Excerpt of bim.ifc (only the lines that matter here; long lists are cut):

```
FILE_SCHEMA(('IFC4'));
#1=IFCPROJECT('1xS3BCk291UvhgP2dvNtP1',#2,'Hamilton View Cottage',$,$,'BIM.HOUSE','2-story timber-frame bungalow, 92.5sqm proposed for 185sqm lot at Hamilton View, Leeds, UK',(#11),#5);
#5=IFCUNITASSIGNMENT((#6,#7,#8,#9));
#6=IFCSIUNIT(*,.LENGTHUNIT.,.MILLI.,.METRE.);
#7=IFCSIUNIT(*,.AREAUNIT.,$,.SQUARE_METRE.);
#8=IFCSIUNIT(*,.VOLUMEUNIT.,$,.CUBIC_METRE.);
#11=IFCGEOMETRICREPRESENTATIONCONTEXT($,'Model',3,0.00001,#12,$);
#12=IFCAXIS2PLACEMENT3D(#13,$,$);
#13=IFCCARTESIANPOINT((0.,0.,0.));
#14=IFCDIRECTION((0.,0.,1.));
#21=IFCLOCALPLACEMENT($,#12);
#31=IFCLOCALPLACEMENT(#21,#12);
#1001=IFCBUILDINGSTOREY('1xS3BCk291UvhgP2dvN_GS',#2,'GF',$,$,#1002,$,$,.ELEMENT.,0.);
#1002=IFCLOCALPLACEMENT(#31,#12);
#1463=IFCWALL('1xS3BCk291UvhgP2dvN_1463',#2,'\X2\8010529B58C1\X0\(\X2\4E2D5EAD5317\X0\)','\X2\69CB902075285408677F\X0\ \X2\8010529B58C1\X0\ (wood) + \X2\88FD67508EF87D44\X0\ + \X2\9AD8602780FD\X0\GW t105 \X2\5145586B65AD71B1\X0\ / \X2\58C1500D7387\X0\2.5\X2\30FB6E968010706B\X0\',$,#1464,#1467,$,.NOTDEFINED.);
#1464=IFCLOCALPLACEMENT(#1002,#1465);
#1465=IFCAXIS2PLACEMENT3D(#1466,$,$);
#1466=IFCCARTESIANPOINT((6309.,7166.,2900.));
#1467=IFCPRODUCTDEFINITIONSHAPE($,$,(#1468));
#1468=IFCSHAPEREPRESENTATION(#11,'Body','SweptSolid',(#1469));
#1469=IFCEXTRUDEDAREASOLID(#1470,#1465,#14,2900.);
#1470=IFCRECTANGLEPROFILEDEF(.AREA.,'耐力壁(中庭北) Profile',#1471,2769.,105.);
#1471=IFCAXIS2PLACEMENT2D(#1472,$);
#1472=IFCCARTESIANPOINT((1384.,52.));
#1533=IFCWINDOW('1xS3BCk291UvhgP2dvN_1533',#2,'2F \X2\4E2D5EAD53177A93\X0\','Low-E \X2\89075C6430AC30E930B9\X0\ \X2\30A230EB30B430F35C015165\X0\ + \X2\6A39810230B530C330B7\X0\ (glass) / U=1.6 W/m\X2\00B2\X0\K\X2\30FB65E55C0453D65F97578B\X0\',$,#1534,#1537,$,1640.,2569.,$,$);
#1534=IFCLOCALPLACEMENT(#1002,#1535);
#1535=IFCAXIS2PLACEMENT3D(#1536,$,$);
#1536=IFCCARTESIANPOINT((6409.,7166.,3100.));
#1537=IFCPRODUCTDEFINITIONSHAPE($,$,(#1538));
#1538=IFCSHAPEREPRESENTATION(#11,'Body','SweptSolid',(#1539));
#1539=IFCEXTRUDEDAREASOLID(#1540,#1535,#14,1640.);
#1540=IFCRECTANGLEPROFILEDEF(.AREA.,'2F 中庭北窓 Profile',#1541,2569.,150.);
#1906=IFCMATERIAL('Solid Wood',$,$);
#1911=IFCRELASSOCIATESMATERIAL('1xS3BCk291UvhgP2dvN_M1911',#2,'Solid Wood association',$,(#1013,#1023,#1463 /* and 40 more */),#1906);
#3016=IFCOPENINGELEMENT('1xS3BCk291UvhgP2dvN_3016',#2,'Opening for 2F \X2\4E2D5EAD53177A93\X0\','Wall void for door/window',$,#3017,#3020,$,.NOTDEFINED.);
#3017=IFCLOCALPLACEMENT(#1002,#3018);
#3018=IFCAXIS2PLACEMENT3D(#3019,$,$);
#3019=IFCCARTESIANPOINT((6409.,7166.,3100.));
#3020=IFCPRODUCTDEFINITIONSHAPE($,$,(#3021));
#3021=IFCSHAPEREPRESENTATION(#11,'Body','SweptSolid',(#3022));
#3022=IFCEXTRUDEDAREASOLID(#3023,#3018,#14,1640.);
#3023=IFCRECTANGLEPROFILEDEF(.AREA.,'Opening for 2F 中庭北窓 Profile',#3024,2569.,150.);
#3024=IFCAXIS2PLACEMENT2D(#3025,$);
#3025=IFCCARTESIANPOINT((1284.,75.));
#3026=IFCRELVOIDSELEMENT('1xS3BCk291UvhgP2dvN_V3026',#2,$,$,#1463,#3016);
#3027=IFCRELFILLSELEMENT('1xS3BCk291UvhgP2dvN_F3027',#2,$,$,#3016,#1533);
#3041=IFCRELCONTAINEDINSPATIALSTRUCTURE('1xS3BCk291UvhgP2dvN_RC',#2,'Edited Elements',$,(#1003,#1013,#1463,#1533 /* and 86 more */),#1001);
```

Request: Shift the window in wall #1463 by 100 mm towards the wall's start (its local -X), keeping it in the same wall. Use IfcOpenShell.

```python
import ifcopenshell
import ifcopenshell.api.geometry
import ifcopenshell.util.placement
import ifcopenshell.util.unit

model = ifcopenshell.open("bim.ifc")
unit_scale = ifcopenshell.util.unit.calculate_unit_scale(model)

window = model.by_id(1533)
opening = window.FillsVoids[0].RelatingOpeningElement
wall = opening.VoidsElements[0].RelatingBuildingElement

wall_matrix = ifcopenshell.util.placement.get_local_placement(wall.ObjectPlacement)
shift = wall_matrix[:3, 0] * -0.1 / unit_scale
before = ifcopenshell.util.placement.get_local_placement(window.ObjectPlacement)[:3, 3].copy()

# The window is not placed relative to its opening, so move both.
for product in (opening, window):
    matrix = ifcopenshell.util.placement.get_local_placement(product.ObjectPlacement)
    matrix[:3, 3] += shift
    ifcopenshell.api.geometry.edit_object_placement(model, product=product, matrix=matrix, is_si=False)

after = ifcopenshell.util.placement.get_local_placement(window.ObjectPlacement)[:3, 3]
print("window moved by", (after - before).round(3) + 0.0)

model.write("bim_rev.ifc")
```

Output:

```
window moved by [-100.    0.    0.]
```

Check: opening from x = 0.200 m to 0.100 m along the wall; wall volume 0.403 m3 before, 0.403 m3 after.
